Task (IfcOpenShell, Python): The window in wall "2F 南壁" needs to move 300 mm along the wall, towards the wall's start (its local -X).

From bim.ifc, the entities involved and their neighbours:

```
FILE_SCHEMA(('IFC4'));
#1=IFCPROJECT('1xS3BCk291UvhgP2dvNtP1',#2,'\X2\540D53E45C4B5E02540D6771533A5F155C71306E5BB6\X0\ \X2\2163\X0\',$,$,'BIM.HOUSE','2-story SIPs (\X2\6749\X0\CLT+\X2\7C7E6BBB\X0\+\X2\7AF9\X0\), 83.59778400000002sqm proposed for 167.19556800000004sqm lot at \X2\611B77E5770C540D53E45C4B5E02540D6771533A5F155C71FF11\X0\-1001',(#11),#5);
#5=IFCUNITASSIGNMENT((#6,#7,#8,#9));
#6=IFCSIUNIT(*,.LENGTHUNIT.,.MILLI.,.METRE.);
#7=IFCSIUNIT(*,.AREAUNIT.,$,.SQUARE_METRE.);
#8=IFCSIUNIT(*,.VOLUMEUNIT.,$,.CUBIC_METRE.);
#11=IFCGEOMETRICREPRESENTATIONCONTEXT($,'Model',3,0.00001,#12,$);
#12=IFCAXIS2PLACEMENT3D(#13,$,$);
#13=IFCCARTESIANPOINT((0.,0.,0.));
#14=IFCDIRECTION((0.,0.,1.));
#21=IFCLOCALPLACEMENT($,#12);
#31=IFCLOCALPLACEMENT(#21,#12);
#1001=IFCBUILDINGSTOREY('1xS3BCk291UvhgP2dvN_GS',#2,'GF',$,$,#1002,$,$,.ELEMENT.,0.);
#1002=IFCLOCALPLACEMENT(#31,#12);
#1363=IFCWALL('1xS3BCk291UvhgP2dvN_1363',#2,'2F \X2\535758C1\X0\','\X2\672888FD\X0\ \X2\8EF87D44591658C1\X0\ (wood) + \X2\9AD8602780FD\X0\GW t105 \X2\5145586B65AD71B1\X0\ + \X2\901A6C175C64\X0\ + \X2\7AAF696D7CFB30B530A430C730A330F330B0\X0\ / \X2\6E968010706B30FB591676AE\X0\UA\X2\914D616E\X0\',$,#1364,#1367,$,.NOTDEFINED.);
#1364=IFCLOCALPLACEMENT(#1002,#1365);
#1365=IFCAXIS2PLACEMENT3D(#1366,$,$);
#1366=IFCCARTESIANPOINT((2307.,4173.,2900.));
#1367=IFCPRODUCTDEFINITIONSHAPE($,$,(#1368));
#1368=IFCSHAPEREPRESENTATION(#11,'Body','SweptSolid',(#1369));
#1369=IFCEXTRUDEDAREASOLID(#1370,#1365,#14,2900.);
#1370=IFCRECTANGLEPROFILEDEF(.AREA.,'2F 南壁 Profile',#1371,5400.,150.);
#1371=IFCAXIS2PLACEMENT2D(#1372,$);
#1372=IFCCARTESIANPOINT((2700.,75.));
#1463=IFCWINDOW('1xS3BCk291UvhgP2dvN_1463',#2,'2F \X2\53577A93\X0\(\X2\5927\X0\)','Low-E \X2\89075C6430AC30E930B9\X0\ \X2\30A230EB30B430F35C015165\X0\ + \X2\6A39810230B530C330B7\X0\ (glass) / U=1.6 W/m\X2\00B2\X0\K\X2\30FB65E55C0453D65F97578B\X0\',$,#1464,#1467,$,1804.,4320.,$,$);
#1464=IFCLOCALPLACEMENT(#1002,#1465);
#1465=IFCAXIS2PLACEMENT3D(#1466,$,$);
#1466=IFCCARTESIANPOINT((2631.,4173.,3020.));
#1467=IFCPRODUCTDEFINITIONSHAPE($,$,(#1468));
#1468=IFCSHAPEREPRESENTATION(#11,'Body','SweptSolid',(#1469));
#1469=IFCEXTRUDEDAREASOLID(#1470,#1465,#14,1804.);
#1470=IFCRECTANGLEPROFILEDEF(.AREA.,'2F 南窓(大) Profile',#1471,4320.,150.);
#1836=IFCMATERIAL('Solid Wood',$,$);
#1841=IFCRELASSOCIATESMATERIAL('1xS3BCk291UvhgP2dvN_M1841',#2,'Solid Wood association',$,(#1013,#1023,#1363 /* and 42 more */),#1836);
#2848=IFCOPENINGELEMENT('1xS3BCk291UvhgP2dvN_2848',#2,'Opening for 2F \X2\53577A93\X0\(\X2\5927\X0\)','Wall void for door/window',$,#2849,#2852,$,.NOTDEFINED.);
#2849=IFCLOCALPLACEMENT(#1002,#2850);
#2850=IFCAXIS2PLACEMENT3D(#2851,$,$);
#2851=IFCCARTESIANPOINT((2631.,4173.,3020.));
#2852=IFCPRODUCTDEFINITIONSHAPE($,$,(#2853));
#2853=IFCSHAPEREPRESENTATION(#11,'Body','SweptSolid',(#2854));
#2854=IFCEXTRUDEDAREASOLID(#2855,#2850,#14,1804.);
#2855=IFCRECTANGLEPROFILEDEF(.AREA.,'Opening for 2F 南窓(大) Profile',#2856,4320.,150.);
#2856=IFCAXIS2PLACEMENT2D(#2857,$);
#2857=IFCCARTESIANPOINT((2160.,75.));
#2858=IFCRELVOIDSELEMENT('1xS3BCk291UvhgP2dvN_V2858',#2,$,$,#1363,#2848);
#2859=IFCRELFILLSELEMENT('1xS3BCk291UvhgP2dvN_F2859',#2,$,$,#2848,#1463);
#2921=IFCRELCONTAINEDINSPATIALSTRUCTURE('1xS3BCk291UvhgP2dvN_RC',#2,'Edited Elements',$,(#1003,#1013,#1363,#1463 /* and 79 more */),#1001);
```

```python
import ifcopenshell
import ifcopenshell.api.geometry
import ifcopenshell.util.placement

model = ifcopenshell.open("bim.ifc")

window = model.by_guid("1xS3BCk291UvhgP2dvN_1463")
opening = window.FillsVoids[0].RelatingOpeningElement
wall = opening.VoidsElements[0].RelatingBuildingElement

wall_matrix = ifcopenshell.util.placement.get_local_placement(wall.ObjectPlacement)
shift = wall_matrix[:3, 0] * -300.0
before = ifcopenshell.util.placement.get_local_placement(window.ObjectPlacement)[:3, 3].copy()

# The window is not placed relative to its opening, so move both.
for product in (opening, window):
    matrix = ifcopenshell.util.placement.get_local_placement(product.ObjectPlacement)
    matrix[:3, 3] += shift
    ifcopenshell.api.geometry.edit_object_placement(model, product=product, matrix=matrix, is_si=False)

after = ifcopenshell.util.placement.get_local_placement(window.ObjectPlacement)[:3, 3]
print("window moved by", (after - before).round(3) + 0.0)

model.write("bim_rev.ifc")
```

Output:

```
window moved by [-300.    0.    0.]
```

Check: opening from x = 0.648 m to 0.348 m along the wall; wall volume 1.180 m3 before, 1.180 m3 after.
